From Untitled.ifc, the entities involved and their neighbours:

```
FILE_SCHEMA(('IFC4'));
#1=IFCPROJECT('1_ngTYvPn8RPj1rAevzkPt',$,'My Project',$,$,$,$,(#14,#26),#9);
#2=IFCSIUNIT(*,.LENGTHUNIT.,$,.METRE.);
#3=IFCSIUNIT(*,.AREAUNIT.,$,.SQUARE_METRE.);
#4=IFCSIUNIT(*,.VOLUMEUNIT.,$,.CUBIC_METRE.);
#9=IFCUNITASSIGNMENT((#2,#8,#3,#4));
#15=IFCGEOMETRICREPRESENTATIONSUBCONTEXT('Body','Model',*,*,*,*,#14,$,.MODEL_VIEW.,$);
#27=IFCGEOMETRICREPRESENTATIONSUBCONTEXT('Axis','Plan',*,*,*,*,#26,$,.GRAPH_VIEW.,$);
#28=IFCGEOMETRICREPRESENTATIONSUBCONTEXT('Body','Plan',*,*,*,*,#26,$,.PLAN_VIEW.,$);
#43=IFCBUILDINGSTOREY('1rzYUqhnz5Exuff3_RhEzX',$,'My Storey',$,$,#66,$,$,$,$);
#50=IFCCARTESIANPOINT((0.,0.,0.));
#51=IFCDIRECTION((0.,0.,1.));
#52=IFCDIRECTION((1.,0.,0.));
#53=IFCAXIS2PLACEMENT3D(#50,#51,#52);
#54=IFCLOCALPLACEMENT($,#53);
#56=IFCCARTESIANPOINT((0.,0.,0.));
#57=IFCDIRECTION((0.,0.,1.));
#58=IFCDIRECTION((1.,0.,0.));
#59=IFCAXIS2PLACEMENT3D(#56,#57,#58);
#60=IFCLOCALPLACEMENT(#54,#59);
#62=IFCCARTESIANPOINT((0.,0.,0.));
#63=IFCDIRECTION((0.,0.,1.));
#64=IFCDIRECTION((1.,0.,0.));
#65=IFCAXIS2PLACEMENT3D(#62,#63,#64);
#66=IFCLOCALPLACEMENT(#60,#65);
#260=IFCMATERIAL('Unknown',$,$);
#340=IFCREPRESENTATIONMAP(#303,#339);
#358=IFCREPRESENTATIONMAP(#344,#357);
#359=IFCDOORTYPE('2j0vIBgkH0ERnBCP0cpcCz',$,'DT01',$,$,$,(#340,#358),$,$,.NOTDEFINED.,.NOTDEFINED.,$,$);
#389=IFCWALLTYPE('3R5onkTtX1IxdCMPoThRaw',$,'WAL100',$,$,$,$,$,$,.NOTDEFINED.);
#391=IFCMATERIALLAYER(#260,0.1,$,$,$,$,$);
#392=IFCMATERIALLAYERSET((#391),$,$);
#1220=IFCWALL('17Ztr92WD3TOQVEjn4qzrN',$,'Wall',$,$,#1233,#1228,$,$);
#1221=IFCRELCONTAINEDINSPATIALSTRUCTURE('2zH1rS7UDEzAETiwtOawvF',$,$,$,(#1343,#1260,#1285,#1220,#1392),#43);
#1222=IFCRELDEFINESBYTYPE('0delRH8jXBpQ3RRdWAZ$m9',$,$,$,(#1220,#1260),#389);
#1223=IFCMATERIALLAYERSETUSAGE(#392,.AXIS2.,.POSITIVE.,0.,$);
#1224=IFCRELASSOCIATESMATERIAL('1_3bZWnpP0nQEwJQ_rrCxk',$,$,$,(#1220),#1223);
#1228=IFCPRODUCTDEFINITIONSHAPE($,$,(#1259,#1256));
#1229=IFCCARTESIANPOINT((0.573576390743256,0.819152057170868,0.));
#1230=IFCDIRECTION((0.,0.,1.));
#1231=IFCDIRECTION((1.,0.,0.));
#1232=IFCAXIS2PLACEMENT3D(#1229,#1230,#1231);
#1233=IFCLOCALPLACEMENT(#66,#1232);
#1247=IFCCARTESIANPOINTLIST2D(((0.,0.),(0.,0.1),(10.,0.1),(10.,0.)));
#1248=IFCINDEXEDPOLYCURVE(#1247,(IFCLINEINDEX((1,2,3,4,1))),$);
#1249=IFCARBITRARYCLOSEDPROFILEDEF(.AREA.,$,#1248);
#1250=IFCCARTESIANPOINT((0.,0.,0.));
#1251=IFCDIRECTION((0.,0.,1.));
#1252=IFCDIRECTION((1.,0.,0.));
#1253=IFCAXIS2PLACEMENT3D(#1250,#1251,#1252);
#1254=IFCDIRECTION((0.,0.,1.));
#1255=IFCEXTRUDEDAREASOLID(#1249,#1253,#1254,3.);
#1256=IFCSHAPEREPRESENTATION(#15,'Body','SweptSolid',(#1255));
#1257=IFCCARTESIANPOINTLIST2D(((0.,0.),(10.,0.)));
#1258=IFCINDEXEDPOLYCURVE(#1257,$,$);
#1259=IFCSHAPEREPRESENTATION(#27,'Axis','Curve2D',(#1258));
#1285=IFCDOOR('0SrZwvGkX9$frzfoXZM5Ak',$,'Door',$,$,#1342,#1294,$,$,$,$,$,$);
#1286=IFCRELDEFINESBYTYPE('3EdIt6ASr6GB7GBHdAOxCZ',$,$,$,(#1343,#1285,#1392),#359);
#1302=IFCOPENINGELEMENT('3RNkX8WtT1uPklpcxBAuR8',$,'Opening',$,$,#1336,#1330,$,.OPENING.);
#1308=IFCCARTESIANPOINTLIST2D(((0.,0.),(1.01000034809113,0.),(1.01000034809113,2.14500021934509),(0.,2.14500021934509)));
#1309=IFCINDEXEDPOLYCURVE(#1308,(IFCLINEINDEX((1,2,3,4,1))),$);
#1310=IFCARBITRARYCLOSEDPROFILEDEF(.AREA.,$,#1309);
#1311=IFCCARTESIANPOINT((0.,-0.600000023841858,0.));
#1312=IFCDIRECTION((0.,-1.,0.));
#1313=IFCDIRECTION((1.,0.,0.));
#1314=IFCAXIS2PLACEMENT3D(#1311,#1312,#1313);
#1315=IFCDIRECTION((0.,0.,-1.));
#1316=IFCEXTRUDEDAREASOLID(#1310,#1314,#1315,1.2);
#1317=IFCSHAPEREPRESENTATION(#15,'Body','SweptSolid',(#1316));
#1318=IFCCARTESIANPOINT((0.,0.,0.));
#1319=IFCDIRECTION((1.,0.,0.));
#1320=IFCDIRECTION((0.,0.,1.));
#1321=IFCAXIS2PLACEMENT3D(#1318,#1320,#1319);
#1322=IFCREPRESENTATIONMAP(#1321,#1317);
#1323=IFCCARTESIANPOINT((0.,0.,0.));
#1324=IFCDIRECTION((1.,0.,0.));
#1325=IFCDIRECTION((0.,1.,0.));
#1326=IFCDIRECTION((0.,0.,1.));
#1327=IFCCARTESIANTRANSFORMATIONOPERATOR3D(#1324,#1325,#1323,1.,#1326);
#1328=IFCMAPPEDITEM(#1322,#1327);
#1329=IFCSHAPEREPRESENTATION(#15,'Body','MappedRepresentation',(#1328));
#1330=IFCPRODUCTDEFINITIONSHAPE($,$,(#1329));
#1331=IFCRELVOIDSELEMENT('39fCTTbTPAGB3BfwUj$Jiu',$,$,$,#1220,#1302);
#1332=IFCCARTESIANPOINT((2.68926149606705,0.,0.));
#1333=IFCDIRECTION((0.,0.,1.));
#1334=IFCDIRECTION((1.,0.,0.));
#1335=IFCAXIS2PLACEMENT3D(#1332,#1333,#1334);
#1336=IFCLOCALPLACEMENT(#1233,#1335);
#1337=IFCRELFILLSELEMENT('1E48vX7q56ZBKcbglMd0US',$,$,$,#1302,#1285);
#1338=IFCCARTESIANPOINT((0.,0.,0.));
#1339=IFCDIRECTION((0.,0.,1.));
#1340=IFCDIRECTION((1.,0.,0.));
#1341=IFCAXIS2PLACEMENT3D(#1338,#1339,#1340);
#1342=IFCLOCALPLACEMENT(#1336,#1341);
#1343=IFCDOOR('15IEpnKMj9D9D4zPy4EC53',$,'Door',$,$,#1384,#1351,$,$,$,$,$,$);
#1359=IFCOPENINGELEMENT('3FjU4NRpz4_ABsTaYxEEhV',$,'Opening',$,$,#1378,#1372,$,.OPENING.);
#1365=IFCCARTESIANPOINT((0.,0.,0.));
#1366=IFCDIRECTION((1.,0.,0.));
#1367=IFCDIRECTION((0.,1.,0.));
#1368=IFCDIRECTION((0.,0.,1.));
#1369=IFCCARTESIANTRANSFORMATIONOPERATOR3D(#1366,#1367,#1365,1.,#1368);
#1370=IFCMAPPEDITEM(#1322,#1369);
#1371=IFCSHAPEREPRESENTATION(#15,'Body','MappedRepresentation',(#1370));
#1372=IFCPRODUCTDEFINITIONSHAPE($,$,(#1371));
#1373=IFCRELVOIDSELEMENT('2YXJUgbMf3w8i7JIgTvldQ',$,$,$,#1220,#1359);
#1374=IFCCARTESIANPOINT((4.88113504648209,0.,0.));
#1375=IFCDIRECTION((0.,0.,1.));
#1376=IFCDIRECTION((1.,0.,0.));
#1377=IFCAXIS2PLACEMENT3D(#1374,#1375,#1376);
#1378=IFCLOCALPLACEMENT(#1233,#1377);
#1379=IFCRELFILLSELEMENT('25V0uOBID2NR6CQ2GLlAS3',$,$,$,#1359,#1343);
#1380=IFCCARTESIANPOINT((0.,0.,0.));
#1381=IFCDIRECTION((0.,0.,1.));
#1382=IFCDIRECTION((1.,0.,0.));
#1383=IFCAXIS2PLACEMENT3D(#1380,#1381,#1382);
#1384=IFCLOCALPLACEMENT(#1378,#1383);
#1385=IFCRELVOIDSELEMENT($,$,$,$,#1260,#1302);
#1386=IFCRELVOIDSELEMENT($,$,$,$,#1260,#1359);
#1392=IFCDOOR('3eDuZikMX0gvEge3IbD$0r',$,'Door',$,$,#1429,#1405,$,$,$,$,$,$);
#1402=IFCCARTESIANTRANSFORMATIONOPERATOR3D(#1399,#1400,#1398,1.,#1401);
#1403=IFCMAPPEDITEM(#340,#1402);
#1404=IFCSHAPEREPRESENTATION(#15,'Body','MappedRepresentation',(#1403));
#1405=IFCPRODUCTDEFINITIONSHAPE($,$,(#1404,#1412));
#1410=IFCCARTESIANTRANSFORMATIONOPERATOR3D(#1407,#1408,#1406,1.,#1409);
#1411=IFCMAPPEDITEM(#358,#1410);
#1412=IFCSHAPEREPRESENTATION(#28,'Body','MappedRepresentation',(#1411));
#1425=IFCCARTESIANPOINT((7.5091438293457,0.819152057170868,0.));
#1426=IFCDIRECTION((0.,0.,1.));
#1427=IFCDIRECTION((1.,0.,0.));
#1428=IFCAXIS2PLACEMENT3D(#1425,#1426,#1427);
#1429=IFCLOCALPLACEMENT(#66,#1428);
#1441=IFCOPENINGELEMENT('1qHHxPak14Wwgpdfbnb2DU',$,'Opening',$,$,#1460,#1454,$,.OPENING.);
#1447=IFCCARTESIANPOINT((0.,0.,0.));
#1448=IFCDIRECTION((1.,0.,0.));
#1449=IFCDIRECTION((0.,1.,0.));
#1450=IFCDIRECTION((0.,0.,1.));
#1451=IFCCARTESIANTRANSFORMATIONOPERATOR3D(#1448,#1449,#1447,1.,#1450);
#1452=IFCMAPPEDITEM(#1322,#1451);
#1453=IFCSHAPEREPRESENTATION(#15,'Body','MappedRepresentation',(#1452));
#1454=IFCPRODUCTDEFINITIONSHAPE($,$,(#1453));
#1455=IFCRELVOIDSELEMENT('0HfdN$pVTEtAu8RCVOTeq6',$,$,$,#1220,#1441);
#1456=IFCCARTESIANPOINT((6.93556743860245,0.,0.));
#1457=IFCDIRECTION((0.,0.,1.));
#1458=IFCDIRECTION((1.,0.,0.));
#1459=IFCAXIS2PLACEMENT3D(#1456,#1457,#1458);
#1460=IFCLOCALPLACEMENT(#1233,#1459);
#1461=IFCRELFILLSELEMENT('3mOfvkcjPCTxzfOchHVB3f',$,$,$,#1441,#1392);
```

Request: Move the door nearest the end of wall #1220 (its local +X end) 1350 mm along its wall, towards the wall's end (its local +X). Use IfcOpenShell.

```python
import ifcopenshell
import ifcopenshell.api.geometry
import ifcopenshell.util.placement
import ifcopenshell.util.unit

model = ifcopenshell.open("Untitled.ifc")
unit_scale = ifcopenshell.util.unit.calculate_unit_scale(model)

door = model.by_guid("3eDuZikMX0gvEge3IbD$0r")
opening = door.FillsVoids[0].RelatingOpeningElement
wall = opening.VoidsElements[0].RelatingBuildingElement

wall_matrix = ifcopenshell.util.placement.get_local_placement(wall.ObjectPlacement)
shift = wall_matrix[:3, 0] * 1.35 / unit_scale
before = ifcopenshell.util.placement.get_local_placement(door.ObjectPlacement)[:3, 3].copy()

# The door is not placed relative to its opening, so move both.
for product in (opening, door):
    matrix = ifcopenshell.util.placement.get_local_placement(product.ObjectPlacement)
    matrix[:3, 3] += shift
    ifcopenshell.api.geometry.edit_object_placement(model, product=product, matrix=matrix, is_si=False)

after = ifcopenshell.util.placement.get_local_placement(door.ObjectPlacement)[:3, 3]
print("door moved by", (after - before).round(3) + 0.0)

model.write("Untitled_updated.ifc")
```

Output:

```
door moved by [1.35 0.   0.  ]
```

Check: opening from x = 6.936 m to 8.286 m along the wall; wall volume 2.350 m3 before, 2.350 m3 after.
